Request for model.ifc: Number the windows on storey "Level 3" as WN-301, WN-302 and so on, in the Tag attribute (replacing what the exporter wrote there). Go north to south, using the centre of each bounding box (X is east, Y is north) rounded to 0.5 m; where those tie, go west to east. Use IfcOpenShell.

First a look at what the model holds.

```python
import ifcopenshell
import ifcopenshell.util.element
import ifcopenshell.util.placement

model = ifcopenshell.open("model.ifc")
print(model.schema)
storey = next(s for s in model.by_type("IfcBuildingStorey") if s.Name == "Level 3")
windows = [e for e in ifcopenshell.util.element.get_decomposition(storey) if e.is_a("IfcWindow")]
for e in sorted(windows, key=lambda e: e.id()):
    origin = ifcopenshell.util.placement.get_local_placement(e.ObjectPlacement)[:3, 3]
    print(e.id(), e.Tag, e.Name, origin.round(2) + 0.0, sep=" | ")
```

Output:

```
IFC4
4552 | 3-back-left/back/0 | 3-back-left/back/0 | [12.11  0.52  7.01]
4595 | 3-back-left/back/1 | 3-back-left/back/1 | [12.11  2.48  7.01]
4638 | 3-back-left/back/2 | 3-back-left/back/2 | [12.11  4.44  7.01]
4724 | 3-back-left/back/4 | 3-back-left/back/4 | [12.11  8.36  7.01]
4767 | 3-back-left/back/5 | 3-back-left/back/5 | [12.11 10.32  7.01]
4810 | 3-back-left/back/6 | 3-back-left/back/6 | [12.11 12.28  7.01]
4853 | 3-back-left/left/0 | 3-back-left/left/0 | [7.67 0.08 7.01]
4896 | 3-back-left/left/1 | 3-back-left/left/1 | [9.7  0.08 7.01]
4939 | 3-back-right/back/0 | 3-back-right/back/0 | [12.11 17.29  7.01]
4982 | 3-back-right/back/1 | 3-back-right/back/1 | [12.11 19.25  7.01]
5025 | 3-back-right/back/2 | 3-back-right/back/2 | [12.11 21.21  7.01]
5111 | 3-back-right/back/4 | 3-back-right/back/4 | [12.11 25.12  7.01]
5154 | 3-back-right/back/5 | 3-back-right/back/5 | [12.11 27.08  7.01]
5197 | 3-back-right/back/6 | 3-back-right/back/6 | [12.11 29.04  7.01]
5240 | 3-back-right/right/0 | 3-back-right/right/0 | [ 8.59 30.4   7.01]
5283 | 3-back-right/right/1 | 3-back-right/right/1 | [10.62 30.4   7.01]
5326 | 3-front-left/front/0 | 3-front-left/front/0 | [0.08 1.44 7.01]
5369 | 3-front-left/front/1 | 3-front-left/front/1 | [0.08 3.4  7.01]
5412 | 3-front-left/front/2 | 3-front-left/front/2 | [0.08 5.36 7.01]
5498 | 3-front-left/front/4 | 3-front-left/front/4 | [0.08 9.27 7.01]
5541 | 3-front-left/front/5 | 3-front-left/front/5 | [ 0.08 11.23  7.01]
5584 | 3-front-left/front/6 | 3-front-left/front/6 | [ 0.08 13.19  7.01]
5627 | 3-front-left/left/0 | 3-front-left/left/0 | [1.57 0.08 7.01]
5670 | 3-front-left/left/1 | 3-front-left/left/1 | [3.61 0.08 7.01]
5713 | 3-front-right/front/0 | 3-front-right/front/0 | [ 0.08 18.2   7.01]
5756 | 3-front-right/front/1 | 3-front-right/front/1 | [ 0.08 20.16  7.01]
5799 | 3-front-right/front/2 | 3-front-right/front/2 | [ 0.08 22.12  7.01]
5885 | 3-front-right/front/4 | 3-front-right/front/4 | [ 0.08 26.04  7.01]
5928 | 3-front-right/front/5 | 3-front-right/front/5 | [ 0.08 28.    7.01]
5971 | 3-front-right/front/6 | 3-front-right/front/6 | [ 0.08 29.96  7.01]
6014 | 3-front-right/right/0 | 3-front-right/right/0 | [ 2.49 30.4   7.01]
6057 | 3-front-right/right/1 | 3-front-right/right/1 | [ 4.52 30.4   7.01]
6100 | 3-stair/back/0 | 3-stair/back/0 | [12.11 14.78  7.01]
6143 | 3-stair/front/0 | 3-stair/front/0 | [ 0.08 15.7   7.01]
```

```python
import ifcopenshell
import ifcopenshell.geom
import ifcopenshell.util.element
import ifcopenshell.util.shape

model = ifcopenshell.open("model.ifc")
settings = ifcopenshell.geom.settings()
settings.set("use-world-coords", True)


def centre(element):
    shape = ifcopenshell.geom.create_shape(settings, element)
    return ifcopenshell.util.shape.get_bbox_centroid(shape.geometry)


storey = next(s for s in model.by_type("IfcBuildingStorey") if s.Name == "Level 3")
windows = [e for e in ifcopenshell.util.element.get_decomposition(storey) if e.is_a("IfcWindow")]

# Insertion points can sit at a corner or the storey origin, so sort by the geometry (in metres).
centres = {e: centre(e) for e in windows}
windows.sort(key=lambda e: (-round(centres[e][1] / 0.5), centres[e][0]))

for i, e in enumerate(windows, start=1):
    number = f"WN-3{i:02d}"
    e.Tag = number
    print(e.id(), number)

model.write("model-out.ifc")
```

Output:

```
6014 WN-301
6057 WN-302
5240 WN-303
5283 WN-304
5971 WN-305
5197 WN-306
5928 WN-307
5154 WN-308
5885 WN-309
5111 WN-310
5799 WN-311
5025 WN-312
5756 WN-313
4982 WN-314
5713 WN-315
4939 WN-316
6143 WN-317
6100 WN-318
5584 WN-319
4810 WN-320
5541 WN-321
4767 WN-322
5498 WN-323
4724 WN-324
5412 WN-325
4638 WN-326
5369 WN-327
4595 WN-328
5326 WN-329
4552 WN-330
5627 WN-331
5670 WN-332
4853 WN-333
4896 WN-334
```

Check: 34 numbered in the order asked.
